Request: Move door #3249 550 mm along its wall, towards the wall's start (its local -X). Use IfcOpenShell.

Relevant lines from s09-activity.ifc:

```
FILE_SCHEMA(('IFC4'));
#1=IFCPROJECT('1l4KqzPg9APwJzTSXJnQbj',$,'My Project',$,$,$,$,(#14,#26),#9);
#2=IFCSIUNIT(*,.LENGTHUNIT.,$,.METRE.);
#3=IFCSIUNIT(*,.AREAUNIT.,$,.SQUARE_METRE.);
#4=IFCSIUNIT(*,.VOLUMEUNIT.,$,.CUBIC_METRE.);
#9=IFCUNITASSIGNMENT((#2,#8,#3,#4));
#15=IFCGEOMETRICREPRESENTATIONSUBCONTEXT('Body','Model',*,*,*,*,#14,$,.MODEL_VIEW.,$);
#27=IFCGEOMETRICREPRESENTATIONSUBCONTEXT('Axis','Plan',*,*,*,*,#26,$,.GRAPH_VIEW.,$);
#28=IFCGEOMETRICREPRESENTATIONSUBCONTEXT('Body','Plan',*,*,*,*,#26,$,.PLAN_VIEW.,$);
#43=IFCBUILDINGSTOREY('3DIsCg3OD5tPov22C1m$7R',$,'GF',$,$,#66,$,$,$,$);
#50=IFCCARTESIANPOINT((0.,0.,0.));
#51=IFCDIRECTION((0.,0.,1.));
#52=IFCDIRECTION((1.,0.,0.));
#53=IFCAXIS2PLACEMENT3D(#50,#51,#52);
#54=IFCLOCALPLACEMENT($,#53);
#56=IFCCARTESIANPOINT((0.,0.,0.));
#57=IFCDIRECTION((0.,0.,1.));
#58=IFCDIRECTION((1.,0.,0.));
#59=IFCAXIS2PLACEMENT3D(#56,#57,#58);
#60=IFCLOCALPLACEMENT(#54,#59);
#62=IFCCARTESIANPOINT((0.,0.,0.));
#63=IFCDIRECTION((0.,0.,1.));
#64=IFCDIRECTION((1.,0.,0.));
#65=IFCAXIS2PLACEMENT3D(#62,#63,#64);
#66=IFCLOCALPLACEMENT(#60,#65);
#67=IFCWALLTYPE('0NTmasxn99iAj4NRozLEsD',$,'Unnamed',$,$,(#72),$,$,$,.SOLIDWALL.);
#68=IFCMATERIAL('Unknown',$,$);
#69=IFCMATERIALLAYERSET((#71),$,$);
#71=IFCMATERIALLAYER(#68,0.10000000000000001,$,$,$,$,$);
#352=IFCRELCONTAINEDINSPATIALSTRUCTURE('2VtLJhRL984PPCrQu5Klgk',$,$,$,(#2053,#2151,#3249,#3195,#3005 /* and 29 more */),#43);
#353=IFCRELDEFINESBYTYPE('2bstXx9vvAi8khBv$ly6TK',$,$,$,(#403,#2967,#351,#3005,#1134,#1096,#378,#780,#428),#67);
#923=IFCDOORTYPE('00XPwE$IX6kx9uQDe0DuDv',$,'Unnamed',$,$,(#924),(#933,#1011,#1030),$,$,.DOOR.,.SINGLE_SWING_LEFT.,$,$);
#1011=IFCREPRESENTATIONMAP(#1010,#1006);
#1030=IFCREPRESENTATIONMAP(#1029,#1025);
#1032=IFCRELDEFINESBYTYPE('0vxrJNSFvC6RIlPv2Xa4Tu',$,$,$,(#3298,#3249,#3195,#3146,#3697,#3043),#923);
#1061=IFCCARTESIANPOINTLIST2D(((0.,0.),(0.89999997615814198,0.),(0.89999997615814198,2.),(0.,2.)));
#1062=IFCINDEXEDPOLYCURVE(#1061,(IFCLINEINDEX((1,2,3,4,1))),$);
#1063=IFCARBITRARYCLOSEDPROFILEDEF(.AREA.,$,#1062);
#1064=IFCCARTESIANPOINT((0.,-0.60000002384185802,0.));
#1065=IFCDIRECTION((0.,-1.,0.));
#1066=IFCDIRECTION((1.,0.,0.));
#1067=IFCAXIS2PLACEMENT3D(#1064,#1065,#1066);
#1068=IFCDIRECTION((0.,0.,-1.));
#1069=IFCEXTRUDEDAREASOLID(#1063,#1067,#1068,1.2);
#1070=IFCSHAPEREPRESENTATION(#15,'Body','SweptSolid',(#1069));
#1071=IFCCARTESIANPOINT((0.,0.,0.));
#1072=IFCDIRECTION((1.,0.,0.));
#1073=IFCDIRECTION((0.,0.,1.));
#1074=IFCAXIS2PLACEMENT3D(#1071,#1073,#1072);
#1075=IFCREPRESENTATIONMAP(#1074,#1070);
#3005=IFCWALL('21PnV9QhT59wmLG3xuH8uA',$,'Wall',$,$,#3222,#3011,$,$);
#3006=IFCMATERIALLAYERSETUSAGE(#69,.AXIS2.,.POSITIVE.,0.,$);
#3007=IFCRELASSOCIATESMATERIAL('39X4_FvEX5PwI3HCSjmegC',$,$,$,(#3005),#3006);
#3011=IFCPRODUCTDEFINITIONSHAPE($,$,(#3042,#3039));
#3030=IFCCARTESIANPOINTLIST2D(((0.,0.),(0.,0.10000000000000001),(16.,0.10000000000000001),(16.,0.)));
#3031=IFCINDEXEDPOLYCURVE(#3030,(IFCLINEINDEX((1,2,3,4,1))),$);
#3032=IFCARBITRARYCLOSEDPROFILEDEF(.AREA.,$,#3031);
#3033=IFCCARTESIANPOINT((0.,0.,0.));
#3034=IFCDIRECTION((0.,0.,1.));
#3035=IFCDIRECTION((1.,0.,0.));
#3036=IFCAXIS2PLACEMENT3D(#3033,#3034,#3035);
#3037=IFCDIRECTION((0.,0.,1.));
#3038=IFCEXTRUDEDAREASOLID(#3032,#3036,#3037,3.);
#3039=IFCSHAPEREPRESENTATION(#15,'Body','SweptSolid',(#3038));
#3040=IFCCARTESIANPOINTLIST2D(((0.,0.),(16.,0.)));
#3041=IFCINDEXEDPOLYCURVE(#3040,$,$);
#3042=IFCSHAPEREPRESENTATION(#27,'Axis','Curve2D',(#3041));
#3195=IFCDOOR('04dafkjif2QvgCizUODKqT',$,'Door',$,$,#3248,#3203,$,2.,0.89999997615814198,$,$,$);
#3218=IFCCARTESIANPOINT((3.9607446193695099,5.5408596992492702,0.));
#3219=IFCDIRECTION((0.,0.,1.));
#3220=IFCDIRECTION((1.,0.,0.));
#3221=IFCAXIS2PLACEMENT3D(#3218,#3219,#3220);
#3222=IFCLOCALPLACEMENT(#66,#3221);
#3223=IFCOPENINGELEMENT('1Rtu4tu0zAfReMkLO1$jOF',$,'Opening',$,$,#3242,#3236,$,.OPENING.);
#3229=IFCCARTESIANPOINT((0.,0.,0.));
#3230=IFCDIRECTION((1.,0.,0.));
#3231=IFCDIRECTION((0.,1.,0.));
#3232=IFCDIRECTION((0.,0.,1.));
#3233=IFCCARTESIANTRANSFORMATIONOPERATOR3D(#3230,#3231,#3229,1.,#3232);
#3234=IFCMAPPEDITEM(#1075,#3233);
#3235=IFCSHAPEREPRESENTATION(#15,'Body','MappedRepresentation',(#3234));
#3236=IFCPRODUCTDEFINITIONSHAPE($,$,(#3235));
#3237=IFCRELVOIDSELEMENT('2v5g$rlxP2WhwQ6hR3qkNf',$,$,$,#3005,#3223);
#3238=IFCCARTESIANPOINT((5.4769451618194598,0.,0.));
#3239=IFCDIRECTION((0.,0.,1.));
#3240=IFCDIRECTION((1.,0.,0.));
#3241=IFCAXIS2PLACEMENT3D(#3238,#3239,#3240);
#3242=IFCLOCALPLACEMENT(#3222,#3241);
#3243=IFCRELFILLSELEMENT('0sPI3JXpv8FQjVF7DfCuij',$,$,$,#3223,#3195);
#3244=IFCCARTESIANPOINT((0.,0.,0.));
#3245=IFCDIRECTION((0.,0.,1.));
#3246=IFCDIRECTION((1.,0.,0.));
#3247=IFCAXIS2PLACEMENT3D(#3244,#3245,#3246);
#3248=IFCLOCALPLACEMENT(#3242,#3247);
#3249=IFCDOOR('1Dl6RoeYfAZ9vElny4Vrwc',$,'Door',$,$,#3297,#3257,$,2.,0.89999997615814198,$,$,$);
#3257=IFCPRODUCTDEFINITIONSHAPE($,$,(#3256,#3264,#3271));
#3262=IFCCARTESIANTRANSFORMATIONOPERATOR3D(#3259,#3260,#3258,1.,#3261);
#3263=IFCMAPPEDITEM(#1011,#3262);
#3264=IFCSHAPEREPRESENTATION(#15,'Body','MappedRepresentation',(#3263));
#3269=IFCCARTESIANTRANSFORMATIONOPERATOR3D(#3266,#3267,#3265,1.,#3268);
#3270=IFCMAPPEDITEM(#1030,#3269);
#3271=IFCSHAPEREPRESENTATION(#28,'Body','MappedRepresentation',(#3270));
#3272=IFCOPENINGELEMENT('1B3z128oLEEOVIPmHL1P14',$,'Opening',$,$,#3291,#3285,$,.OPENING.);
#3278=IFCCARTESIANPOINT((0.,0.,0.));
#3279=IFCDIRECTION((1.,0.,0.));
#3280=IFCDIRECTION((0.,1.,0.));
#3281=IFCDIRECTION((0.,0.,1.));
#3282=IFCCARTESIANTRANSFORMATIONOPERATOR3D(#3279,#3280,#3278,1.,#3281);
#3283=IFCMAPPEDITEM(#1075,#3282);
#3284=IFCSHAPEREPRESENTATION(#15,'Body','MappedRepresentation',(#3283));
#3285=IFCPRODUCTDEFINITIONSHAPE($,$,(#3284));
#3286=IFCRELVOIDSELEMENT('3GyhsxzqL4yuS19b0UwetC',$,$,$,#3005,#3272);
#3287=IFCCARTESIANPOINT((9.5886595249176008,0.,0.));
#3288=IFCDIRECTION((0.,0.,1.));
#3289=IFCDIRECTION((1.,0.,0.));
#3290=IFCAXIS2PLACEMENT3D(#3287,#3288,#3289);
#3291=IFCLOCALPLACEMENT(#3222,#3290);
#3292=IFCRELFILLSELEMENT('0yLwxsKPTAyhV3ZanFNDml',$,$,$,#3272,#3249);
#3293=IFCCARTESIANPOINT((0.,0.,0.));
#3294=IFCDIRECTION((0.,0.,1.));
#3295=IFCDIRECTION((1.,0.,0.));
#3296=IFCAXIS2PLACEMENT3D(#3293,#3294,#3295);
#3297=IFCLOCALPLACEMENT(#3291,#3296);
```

```python
import ifcopenshell
import ifcopenshell.api.geometry
import ifcopenshell.util.placement
import ifcopenshell.util.unit

model = ifcopenshell.open("s09-activity.ifc")
unit_scale = ifcopenshell.util.unit.calculate_unit_scale(model)

door = model.by_guid("1Dl6RoeYfAZ9vElny4Vrwc")
opening = door.FillsVoids[0].RelatingOpeningElement
wall = opening.VoidsElements[0].RelatingBuildingElement

wall_matrix = ifcopenshell.util.placement.get_local_placement(wall.ObjectPlacement)
shift = wall_matrix[:3, 0] * -0.55 / unit_scale
before = ifcopenshell.util.placement.get_local_placement(door.ObjectPlacement)[:3, 3].copy()

# The door is placed relative to its opening, so it follows when the opening moves.
matrix = ifcopenshell.util.placement.get_local_placement(opening.ObjectPlacement)
matrix[:3, 3] += shift
ifcopenshell.api.geometry.edit_object_placement(
    model, product=opening, matrix=matrix, is_si=False, should_transform_children=True
)

after = ifcopenshell.util.placement.get_local_placement(door.ObjectPlacement)[:3, 3]
print("door moved by", (after - before).round(3) + 0.0)

model.write("s09-activity_updated.ifc")
```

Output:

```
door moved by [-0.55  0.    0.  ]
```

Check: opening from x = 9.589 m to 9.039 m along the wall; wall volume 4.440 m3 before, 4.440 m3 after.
